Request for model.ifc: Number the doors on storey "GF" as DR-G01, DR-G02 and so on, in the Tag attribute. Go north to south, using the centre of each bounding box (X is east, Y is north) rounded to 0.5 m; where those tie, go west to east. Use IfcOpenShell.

First a look at what the model holds.

```python
import ifcopenshell
import ifcopenshell.util.element
import ifcopenshell.util.placement

model = ifcopenshell.open("model.ifc")
print(model.schema)
storey = next(s for s in model.by_type("IfcBuildingStorey") if s.Name == "GF")
doors = [e for e in ifcopenshell.util.element.get_decomposition(storey) if e.is_a("IfcDoor")]
for e in sorted(doors, key=lambda e: e.id()):
    origin = ifcopenshell.util.placement.get_local_placement(e.ObjectPlacement)[:3, 3]
    print(e.id(), e.Tag, e.Name, origin.round(2) + 0.0, sep=" | ")
```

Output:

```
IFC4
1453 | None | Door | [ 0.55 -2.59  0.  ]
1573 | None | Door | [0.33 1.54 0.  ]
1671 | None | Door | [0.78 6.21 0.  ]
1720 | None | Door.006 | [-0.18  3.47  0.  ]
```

```python
import ifcopenshell
import ifcopenshell.geom
import ifcopenshell.util.element
import ifcopenshell.util.shape

model = ifcopenshell.open("model.ifc")
settings = ifcopenshell.geom.settings()
settings.set("use-world-coords", True)


def centre(element):
    shape = ifcopenshell.geom.create_shape(settings, element)
    return ifcopenshell.util.shape.get_bbox_centroid(shape.geometry)


storey = next(s for s in model.by_type("IfcBuildingStorey") if s.Name == "GF")
doors = [e for e in ifcopenshell.util.element.get_decomposition(storey) if e.is_a("IfcDoor")]

# Insertion points can sit at a corner or the storey origin, so sort by the geometry (in metres).
centres = {e: centre(e) for e in doors}
doors.sort(key=lambda e: (-round(centres[e][1] / 0.5), centres[e][0]))

for i, e in enumerate(doors, start=1):
    number = f"DR-G{i:02d}"
    e.Tag = number
    print(e.id(), number)

model.write("model_v2.ifc")
```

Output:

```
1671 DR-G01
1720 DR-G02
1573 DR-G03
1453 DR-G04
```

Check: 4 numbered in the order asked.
